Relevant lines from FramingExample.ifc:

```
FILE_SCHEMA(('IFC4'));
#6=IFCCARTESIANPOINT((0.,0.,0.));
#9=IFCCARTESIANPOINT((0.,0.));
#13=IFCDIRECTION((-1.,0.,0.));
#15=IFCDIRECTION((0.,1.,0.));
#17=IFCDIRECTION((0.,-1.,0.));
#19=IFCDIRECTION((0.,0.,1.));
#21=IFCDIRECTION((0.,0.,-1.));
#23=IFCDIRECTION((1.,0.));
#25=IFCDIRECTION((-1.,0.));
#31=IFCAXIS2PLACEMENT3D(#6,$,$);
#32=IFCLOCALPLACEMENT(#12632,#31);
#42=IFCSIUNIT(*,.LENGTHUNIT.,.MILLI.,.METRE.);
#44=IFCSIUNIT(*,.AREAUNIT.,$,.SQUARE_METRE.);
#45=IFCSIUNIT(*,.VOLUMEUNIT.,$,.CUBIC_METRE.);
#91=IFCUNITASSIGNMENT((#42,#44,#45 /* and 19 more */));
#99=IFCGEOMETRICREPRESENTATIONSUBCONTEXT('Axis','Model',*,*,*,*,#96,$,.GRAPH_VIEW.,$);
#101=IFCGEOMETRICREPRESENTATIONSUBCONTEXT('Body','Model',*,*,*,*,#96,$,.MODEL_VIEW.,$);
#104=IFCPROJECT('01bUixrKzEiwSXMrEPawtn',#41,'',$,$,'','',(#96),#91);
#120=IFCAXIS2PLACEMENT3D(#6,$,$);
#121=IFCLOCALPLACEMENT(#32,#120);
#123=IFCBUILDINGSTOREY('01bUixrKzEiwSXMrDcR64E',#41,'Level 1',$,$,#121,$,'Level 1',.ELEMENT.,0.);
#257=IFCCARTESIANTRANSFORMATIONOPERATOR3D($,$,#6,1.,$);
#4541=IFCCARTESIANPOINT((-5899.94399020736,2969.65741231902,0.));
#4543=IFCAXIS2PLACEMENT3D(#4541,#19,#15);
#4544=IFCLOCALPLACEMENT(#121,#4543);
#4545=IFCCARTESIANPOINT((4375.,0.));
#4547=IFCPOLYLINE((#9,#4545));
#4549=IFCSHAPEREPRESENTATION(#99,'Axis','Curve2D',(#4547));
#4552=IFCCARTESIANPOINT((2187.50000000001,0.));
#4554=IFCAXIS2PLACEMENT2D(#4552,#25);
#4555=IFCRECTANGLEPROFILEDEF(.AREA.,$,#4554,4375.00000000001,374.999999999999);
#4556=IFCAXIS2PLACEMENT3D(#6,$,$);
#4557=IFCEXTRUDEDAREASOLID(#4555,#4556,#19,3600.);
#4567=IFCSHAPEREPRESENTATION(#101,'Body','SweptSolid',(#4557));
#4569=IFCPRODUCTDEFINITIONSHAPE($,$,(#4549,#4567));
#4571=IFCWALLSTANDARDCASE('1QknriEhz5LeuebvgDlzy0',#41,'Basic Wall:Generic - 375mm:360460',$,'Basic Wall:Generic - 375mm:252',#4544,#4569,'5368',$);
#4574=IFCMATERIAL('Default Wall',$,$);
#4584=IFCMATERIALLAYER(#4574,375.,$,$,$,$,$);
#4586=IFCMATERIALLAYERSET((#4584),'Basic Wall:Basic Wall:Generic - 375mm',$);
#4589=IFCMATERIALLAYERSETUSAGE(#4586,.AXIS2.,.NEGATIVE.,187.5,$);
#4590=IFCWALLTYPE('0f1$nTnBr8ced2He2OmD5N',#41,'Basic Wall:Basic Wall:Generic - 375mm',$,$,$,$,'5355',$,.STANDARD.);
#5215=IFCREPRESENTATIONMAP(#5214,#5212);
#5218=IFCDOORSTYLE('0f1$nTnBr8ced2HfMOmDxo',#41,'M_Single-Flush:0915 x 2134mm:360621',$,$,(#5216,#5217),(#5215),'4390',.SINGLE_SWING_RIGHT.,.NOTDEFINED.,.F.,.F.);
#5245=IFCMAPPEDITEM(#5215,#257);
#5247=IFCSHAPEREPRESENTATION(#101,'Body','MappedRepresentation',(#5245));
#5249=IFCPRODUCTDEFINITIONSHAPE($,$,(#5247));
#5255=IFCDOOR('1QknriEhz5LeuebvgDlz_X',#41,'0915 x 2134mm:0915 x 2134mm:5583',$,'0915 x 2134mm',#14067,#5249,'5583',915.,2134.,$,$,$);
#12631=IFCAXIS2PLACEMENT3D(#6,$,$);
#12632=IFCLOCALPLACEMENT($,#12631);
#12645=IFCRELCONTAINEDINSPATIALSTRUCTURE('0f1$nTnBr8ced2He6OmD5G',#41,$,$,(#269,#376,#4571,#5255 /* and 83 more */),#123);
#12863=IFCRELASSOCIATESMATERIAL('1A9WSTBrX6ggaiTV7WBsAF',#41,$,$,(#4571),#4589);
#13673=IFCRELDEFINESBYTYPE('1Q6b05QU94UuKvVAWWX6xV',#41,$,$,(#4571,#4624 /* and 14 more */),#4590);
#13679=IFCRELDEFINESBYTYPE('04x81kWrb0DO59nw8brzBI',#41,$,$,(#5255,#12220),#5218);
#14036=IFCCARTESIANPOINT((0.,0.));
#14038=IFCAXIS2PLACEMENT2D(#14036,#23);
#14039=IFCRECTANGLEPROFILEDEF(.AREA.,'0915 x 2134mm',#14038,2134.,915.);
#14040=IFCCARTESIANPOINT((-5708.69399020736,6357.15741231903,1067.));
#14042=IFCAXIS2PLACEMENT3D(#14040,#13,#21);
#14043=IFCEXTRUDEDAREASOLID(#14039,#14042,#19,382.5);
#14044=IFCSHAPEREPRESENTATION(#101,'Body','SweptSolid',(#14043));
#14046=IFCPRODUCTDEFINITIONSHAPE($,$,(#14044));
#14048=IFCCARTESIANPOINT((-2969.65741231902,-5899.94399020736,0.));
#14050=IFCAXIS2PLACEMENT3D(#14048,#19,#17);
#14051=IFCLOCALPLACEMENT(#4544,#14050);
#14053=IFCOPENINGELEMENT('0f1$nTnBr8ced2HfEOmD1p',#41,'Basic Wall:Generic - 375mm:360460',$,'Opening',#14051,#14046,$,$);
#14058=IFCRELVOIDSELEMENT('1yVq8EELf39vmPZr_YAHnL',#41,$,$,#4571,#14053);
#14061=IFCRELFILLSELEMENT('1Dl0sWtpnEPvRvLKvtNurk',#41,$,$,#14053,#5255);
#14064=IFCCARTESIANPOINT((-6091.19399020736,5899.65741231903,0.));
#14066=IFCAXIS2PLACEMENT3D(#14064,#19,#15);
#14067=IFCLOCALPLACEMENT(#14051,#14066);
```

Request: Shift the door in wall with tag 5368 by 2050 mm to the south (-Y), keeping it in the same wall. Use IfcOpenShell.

```python
import ifcopenshell
import ifcopenshell.api.geometry
import ifcopenshell.util.placement
import ifcopenshell.util.unit

model = ifcopenshell.open("FramingExample.ifc")
unit_scale = ifcopenshell.util.unit.calculate_unit_scale(model)

door = model.by_guid("1QknriEhz5LeuebvgDlz_X")
opening = door.FillsVoids[0].RelatingOpeningElement
wall = opening.VoidsElements[0].RelatingBuildingElement

wall_matrix = ifcopenshell.util.placement.get_local_placement(wall.ObjectPlacement)
shift = wall_matrix[:3, 0] * -2.05 / unit_scale
before = ifcopenshell.util.placement.get_local_placement(door.ObjectPlacement)[:3, 3].copy()

# The door is placed relative to its opening, so it follows when the opening moves.
matrix = ifcopenshell.util.placement.get_local_placement(opening.ObjectPlacement)
matrix[:3, 3] += shift
ifcopenshell.api.geometry.edit_object_placement(
    model, product=opening, matrix=matrix, is_si=False, should_transform_children=True
)

after = ifcopenshell.util.placement.get_local_placement(door.ObjectPlacement)[:3, 3]
print("door moved by", (after - before).round(3) + 0.0)

model.write("FramingExample_rev.ifc")
```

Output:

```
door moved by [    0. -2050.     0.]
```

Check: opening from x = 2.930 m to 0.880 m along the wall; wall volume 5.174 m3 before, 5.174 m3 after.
